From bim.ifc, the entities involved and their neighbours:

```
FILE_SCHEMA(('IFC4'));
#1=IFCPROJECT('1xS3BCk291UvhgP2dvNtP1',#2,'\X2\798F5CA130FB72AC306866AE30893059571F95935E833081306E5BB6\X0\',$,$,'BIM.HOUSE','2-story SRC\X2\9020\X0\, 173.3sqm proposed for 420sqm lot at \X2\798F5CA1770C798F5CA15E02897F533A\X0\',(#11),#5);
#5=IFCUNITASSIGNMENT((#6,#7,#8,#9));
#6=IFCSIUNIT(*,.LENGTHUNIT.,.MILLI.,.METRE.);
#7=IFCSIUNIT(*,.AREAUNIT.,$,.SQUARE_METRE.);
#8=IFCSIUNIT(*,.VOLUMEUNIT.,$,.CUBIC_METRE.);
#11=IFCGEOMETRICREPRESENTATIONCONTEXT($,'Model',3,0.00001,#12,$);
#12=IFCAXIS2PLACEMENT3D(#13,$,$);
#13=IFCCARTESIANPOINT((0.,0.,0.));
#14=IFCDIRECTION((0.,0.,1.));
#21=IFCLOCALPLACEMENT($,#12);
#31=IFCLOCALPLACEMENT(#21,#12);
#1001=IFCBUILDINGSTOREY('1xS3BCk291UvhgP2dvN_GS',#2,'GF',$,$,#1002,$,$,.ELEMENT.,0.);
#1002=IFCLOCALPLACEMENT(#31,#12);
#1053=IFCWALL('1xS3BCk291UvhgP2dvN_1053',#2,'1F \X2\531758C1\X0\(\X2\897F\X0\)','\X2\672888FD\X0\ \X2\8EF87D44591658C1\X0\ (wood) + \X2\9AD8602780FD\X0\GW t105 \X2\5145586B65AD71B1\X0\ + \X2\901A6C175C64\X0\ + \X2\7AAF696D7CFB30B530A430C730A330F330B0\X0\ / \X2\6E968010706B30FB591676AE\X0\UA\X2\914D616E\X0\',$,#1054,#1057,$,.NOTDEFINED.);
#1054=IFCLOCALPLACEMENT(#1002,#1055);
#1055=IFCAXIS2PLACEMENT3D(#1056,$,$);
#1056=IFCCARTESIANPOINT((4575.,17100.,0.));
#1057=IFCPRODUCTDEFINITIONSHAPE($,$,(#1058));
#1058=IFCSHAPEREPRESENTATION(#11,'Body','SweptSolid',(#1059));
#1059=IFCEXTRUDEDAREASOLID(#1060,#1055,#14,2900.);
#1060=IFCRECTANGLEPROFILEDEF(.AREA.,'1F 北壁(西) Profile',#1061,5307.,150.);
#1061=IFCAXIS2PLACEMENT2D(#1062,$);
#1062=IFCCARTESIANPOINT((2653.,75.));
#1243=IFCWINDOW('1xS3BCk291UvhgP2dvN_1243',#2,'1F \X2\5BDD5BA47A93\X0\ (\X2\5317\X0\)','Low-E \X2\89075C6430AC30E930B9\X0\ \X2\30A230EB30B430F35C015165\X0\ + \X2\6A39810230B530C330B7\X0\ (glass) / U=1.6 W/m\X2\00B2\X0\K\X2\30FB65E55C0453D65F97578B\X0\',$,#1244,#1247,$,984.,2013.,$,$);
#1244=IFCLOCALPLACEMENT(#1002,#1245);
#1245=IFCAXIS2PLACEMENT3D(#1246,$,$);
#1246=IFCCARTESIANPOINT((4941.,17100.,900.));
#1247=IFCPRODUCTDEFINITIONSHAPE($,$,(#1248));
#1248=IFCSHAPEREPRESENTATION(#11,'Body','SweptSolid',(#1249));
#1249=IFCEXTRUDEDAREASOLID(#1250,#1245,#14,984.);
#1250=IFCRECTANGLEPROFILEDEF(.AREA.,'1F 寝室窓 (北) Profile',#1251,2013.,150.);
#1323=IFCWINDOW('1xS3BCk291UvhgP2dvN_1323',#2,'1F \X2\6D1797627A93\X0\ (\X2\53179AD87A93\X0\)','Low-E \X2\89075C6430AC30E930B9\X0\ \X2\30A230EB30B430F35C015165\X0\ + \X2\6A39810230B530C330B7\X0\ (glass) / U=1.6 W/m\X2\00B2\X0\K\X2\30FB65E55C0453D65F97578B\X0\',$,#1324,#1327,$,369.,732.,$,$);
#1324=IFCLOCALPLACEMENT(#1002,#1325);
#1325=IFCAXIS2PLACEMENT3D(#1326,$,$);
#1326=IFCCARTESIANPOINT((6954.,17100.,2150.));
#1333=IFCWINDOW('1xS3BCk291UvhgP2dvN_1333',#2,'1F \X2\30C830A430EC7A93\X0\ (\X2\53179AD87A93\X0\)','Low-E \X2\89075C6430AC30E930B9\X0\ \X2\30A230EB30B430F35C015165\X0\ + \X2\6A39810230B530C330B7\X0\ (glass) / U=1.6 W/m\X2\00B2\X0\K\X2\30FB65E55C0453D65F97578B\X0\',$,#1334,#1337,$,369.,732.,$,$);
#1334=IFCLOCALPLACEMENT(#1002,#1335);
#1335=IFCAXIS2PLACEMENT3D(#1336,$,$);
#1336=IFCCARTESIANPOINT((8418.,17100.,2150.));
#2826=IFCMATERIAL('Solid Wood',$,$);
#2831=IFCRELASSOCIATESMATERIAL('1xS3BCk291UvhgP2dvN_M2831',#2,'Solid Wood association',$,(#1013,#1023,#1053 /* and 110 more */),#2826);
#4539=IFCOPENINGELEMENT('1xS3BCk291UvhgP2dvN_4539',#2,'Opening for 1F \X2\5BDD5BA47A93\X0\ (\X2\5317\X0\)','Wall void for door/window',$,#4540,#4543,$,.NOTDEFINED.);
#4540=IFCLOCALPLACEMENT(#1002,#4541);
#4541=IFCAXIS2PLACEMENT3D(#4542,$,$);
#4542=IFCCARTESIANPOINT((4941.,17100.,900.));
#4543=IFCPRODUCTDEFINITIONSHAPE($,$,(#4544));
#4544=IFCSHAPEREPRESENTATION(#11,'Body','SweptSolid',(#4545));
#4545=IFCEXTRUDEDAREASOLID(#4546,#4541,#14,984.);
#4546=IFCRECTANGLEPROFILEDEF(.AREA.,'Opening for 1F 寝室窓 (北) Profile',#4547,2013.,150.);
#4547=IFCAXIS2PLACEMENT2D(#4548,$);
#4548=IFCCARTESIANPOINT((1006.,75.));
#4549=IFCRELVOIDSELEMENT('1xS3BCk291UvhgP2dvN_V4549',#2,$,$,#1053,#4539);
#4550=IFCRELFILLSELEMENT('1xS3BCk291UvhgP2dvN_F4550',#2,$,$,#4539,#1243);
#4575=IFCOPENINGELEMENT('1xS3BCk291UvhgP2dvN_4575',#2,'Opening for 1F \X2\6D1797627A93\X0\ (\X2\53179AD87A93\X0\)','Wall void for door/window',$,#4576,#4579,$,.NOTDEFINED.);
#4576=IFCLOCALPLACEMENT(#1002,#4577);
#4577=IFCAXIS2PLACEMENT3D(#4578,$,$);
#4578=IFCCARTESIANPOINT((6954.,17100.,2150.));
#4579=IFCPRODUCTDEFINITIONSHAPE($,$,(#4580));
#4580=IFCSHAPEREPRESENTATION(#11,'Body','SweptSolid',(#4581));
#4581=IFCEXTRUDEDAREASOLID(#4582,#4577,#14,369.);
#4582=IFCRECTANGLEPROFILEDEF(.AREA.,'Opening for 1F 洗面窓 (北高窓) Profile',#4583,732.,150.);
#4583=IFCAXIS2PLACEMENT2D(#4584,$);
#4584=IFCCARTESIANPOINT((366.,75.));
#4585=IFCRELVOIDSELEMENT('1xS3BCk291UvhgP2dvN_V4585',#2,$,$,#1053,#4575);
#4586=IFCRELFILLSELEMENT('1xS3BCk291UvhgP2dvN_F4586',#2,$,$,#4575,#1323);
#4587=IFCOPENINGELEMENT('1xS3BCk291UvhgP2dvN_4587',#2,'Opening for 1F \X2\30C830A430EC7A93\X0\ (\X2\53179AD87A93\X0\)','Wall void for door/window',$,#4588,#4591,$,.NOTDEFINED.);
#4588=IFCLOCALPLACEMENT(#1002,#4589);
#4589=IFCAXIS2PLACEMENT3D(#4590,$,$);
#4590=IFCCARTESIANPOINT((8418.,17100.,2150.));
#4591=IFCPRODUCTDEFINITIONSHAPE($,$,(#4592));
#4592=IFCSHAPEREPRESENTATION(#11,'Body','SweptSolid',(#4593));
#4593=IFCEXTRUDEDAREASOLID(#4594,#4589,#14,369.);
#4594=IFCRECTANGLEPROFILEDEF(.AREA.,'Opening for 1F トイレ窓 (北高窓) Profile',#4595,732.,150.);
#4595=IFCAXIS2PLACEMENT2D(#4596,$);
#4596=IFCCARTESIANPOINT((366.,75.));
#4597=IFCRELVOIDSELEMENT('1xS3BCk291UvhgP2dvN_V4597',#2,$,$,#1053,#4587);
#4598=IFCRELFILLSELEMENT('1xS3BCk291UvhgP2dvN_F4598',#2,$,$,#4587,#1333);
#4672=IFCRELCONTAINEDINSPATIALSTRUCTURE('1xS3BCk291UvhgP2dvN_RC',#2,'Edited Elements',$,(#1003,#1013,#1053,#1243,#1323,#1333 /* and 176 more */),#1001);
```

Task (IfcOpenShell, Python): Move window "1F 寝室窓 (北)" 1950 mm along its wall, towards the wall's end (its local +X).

```python
import ifcopenshell
import ifcopenshell.api.geometry
import ifcopenshell.util.placement
import ifcopenshell.util.unit

model = ifcopenshell.open("bim.ifc")
unit_scale = ifcopenshell.util.unit.calculate_unit_scale(model)

window = model.by_guid("1xS3BCk291UvhgP2dvN_1243")
opening = window.FillsVoids[0].RelatingOpeningElement
wall = opening.VoidsElements[0].RelatingBuildingElement

wall_matrix = ifcopenshell.util.placement.get_local_placement(wall.ObjectPlacement)
shift = wall_matrix[:3, 0] * 1.95 / unit_scale
before = ifcopenshell.util.placement.get_local_placement(window.ObjectPlacement)[:3, 3].copy()

# The window is not placed relative to its opening, so move both.
for product in (opening, window):
    matrix = ifcopenshell.util.placement.get_local_placement(product.ObjectPlacement)
    matrix[:3, 3] += shift
    ifcopenshell.api.geometry.edit_object_placement(model, product=product, matrix=matrix, is_si=False)

after = ifcopenshell.util.placement.get_local_placement(window.ObjectPlacement)[:3, 3]
print("window moved by", (after - before).round(3) + 0.0)

model.write("bim_edited.ifc")
```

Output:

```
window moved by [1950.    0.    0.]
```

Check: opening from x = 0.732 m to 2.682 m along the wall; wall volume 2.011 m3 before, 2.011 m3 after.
